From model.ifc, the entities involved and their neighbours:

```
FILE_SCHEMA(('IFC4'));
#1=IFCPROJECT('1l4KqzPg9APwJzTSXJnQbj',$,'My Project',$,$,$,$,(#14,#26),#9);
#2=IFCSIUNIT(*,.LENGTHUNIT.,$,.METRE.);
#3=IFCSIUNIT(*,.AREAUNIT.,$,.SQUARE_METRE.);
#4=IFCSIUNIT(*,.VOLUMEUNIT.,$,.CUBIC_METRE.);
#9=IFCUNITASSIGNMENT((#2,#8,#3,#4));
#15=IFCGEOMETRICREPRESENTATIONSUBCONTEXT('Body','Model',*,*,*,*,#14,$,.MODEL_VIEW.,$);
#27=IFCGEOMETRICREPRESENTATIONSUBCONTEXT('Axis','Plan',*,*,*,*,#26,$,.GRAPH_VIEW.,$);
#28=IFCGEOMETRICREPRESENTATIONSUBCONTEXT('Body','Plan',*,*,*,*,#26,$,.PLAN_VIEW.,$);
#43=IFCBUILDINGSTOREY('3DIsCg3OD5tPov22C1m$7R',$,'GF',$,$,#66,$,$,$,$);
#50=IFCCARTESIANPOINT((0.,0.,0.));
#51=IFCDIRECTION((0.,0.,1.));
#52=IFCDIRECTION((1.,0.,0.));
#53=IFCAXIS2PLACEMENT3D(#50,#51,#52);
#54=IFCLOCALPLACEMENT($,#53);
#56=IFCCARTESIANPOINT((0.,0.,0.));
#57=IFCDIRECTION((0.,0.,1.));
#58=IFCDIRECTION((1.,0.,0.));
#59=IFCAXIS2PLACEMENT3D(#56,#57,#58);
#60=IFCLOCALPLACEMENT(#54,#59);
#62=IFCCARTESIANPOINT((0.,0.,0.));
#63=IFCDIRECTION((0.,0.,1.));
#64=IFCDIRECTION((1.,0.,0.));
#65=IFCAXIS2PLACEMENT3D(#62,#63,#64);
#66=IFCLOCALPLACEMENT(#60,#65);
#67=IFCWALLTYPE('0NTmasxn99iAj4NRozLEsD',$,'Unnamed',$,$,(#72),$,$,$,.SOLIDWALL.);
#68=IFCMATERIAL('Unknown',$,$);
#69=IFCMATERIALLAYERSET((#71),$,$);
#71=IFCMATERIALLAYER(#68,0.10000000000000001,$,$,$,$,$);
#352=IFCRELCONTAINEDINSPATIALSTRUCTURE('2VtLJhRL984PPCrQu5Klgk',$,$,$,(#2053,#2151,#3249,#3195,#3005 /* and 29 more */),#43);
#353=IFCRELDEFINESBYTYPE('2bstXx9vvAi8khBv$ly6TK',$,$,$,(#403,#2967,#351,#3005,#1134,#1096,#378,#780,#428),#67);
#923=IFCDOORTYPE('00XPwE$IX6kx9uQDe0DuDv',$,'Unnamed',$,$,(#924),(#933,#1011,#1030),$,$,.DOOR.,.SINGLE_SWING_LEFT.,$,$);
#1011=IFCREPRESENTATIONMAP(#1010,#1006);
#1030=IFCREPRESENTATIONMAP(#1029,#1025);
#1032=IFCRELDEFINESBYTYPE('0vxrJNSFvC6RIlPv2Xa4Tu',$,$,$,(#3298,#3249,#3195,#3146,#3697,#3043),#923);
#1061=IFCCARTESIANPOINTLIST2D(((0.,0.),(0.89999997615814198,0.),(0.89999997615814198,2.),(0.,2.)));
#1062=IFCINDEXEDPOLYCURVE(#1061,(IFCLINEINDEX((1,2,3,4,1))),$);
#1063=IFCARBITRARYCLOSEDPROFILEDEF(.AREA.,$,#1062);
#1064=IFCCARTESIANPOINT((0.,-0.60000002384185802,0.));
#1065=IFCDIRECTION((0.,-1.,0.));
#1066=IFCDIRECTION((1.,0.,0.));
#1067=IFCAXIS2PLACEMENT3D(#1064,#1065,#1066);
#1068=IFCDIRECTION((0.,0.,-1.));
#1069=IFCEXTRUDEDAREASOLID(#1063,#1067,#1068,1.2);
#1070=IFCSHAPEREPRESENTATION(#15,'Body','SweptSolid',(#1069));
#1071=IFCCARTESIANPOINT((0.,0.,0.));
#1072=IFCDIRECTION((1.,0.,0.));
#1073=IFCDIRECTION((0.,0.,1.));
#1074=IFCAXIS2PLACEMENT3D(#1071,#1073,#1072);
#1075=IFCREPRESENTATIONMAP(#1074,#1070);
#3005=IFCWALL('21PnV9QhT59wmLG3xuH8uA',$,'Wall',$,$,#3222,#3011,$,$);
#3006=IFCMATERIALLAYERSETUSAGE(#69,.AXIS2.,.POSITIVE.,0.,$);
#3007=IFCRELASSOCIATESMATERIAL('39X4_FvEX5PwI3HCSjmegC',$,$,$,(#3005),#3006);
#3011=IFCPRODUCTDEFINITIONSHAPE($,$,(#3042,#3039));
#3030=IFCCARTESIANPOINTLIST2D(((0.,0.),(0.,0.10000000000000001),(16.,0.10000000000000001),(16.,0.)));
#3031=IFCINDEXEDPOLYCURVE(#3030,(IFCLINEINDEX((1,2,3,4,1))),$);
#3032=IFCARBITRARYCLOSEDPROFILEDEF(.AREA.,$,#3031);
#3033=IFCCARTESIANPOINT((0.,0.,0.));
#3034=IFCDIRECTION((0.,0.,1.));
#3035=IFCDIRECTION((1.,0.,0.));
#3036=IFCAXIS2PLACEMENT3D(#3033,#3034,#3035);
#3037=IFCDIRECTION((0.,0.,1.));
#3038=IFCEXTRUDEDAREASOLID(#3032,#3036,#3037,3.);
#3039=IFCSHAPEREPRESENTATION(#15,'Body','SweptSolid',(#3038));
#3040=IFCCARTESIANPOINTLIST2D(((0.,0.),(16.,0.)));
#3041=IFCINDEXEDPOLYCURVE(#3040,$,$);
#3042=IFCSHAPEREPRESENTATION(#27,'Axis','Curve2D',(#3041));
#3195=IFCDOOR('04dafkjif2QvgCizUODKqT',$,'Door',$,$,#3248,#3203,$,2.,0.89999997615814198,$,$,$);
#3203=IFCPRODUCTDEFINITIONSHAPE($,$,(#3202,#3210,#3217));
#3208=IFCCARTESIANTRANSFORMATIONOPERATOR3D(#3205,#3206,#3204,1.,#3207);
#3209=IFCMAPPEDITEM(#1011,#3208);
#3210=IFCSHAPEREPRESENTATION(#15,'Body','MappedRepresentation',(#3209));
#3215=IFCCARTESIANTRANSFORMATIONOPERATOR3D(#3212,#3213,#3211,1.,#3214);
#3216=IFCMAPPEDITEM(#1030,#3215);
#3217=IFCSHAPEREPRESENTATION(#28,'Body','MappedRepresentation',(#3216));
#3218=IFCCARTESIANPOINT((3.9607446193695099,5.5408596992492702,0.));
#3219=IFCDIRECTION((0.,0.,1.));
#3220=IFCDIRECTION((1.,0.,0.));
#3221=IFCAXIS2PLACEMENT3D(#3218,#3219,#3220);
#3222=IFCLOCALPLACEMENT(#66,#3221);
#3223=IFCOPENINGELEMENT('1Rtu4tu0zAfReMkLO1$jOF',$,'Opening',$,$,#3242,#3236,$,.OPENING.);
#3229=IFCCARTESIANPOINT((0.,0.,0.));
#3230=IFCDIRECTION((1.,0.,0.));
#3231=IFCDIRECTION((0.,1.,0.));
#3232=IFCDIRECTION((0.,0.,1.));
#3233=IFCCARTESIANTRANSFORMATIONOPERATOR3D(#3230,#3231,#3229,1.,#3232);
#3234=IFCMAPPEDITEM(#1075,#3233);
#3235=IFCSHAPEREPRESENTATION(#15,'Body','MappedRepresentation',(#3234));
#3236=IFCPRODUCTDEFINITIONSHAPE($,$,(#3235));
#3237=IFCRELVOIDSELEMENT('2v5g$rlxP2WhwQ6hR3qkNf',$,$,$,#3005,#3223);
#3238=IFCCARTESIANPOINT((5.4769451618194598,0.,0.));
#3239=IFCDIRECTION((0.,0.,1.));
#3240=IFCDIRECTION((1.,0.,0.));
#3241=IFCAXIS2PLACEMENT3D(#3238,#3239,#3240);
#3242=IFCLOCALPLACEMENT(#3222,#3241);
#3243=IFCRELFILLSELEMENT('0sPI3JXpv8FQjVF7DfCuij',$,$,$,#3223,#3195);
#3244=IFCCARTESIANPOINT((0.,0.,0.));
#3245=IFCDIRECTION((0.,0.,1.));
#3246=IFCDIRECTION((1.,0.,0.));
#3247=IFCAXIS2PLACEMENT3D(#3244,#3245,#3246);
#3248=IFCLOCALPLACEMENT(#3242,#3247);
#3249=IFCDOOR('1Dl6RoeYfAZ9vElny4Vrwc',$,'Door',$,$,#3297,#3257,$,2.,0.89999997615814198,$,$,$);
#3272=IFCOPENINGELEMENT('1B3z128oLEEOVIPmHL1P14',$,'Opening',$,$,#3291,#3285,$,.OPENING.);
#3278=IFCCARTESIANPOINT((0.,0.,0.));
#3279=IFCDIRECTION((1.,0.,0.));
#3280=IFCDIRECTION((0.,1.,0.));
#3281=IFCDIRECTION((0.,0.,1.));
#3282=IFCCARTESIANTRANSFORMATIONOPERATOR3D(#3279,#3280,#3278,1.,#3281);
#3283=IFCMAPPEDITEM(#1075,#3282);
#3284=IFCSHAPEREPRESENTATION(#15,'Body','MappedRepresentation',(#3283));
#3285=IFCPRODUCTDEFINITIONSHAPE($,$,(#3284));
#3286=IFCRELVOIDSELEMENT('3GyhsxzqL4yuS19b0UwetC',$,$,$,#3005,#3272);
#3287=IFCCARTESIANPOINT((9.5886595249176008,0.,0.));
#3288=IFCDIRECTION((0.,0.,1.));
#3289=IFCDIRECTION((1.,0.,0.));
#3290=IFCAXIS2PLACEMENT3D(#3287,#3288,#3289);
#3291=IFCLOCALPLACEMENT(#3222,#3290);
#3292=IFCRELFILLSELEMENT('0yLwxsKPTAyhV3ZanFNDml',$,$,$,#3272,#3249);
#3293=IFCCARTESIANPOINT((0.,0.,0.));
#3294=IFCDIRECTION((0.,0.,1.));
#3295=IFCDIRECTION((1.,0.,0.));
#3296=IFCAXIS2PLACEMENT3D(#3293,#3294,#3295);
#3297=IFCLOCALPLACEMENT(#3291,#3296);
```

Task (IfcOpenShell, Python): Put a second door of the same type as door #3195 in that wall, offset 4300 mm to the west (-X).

```python
import ifcopenshell
import ifcopenshell.api.feature
import ifcopenshell.api.geometry
import ifcopenshell.api.root
import ifcopenshell.geom
import ifcopenshell.util.element
import ifcopenshell.util.placement
import ifcopenshell.util.shape
import ifcopenshell.util.unit

model = ifcopenshell.open("model.ifc")
unit_scale = ifcopenshell.util.unit.calculate_unit_scale(model)
settings = ifcopenshell.geom.settings()


def volume(element):
    """Net volume in cubic metres, openings subtracted."""
    shape = ifcopenshell.geom.create_shape(settings, element)
    return ifcopenshell.util.shape.get_volume(shape.geometry)


door = model.by_guid("04dafkjif2QvgCizUODKqT")
opening = door.FillsVoids[0].RelatingOpeningElement
wall = opening.VoidsElements[0].RelatingBuildingElement
before = volume(wall)
shift = ifcopenshell.util.placement.get_local_placement(wall.ObjectPlacement)[:3, 0] * -4.3 / unit_scale

# copy_class copies the void relationship, type, container and properties, but no geometry.
new_opening = ifcopenshell.api.root.copy_class(model, product=opening)
new_opening.Representation = ifcopenshell.util.element.copy_deep(
    model, opening.Representation, exclude=["IfcGeometricRepresentationContext", "IfcRepresentationMap"]
)
new_door = ifcopenshell.api.root.copy_class(model, product=door)
new_door.Representation = ifcopenshell.util.element.copy_deep(
    model, door.Representation, exclude=["IfcGeometricRepresentationContext", "IfcRepresentationMap"]
)
ifcopenshell.api.feature.add_filling(model, opening=new_opening, element=new_door)

for old, new in ((opening, new_opening), (door, new_door)):
    matrix = ifcopenshell.util.placement.get_local_placement(old.ObjectPlacement)
    matrix[:3, 3] += shift
    ifcopenshell.api.geometry.edit_object_placement(model, product=new, matrix=matrix, is_si=False)

after = volume(wall)

print(f"wall volume {before:.3f} -> {after:.3f} m3")

model.write("model-out.ifc")
```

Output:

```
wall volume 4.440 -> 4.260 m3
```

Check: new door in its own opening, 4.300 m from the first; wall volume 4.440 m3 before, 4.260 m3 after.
